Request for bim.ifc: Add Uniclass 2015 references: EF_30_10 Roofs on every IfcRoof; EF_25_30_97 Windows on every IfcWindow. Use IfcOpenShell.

First a look at what the model holds.

```python
import ifcopenshell

model = ifcopenshell.open("bim.ifc")
print(model.schema)
print("classifications:", [c.Name for c in model.by_type("IfcClassification")])
for ifc_class in ("IfcDoor", "IfcRoof", "IfcStair", "IfcWall", "IfcWindow"):
    print(ifc_class, len(model.by_type(ifc_class)))
```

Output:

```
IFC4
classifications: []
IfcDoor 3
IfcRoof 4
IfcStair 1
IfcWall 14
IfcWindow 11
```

```python
import ifcopenshell
import ifcopenshell.api.classification

model = ifcopenshell.open("bim.ifc")

system = ifcopenshell.api.classification.add_classification(model, classification="Uniclass 2015")

codes = {
    "IfcRoof": ("EF_30_10", "Roofs"),
    "IfcWindow": ("EF_25_30_97", "Windows"),
}
for ifc_class, (code, name) in codes.items():
    products = model.by_type(ifc_class)
    ifcopenshell.api.classification.add_reference(
        model, products=products, classification=system, identification=code, name=name
    )
    print(code, len(products))

model.write("bim_updated.ifc")
```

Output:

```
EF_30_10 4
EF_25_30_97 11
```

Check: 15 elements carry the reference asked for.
